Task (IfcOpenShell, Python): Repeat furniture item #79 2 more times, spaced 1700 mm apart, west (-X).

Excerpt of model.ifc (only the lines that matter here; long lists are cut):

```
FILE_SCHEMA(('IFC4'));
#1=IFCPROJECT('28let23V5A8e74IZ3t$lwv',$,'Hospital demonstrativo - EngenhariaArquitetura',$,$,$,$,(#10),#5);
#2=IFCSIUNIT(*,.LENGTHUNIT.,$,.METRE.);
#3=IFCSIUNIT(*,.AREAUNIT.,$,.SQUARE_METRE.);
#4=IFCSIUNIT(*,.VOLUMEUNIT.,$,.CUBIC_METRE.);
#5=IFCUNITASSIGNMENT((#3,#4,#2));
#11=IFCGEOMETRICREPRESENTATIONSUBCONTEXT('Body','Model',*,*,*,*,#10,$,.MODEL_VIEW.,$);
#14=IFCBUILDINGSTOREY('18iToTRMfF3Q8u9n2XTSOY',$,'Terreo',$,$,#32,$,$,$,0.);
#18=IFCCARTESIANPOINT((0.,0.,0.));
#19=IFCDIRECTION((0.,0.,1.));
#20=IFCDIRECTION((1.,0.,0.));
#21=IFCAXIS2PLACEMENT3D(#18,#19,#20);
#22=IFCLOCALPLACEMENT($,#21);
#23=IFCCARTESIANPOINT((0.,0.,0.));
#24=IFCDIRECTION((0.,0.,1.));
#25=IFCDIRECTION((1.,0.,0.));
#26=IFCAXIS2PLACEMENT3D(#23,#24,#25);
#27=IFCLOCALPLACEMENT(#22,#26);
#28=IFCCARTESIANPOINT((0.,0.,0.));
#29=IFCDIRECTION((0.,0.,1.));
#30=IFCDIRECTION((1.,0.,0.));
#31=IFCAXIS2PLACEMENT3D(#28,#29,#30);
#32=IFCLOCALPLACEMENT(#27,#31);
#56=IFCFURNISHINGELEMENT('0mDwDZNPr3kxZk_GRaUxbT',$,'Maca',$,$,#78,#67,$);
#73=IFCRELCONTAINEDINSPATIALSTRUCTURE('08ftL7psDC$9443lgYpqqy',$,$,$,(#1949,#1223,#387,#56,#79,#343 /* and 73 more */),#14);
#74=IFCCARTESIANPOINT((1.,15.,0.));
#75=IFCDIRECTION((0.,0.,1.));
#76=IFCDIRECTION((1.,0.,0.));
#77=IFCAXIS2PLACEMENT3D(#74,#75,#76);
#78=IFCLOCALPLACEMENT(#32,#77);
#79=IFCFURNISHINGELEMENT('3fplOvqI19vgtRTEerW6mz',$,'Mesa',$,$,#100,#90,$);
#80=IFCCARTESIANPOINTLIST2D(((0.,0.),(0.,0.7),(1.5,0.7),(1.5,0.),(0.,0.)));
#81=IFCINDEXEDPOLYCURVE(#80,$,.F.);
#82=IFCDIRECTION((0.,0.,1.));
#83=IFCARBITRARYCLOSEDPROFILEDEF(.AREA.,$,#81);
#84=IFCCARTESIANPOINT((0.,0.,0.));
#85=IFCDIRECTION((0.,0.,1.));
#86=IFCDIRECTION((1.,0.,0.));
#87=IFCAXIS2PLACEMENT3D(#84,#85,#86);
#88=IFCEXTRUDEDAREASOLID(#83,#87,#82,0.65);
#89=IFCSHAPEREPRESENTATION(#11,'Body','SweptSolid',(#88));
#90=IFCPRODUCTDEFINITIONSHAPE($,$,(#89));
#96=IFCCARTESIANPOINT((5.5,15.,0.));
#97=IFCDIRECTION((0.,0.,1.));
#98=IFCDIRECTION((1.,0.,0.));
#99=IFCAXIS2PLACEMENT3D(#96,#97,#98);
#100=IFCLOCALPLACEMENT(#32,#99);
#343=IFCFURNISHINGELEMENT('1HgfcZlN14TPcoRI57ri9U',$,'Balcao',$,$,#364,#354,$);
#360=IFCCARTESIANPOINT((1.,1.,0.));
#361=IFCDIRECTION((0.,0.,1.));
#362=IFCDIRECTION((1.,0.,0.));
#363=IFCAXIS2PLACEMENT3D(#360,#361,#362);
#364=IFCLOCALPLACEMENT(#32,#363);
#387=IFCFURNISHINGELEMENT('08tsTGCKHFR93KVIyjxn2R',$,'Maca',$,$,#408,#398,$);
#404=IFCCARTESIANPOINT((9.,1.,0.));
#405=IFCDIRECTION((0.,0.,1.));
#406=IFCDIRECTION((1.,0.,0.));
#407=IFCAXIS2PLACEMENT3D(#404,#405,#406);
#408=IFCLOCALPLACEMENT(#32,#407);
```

```python
import numpy as np
import ifcopenshell
import ifcopenshell.api.geometry
import ifcopenshell.api.root
import ifcopenshell.util.element
import ifcopenshell.util.placement
import ifcopenshell.util.unit

model = ifcopenshell.open("model.ifc")
unit_scale = ifcopenshell.util.unit.calculate_unit_scale(model)

source = model.by_guid("3fplOvqI19vgtRTEerW6mz")
base = ifcopenshell.util.placement.get_local_placement(source.ObjectPlacement)
step = np.array([-1.0, 0.0, 0.0]) * 1.7 / unit_scale

for i in range(1, 3):
    copy = ifcopenshell.api.root.copy_class(model, product=source)
    copy.Representation = ifcopenshell.util.element.copy_deep(
        model, source.Representation, exclude=["IfcGeometricRepresentationContext", "IfcRepresentationMap"]
    )
    matrix = base.copy()
    matrix[:3, 3] += i * step
    print("added at", matrix[:3, 3].round(3) + 0.0)
    ifcopenshell.api.geometry.edit_object_placement(model, product=copy, matrix=matrix, is_si=False)

model.write("model_updated.ifc")
```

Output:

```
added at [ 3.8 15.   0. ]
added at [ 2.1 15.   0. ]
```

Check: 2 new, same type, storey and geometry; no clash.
